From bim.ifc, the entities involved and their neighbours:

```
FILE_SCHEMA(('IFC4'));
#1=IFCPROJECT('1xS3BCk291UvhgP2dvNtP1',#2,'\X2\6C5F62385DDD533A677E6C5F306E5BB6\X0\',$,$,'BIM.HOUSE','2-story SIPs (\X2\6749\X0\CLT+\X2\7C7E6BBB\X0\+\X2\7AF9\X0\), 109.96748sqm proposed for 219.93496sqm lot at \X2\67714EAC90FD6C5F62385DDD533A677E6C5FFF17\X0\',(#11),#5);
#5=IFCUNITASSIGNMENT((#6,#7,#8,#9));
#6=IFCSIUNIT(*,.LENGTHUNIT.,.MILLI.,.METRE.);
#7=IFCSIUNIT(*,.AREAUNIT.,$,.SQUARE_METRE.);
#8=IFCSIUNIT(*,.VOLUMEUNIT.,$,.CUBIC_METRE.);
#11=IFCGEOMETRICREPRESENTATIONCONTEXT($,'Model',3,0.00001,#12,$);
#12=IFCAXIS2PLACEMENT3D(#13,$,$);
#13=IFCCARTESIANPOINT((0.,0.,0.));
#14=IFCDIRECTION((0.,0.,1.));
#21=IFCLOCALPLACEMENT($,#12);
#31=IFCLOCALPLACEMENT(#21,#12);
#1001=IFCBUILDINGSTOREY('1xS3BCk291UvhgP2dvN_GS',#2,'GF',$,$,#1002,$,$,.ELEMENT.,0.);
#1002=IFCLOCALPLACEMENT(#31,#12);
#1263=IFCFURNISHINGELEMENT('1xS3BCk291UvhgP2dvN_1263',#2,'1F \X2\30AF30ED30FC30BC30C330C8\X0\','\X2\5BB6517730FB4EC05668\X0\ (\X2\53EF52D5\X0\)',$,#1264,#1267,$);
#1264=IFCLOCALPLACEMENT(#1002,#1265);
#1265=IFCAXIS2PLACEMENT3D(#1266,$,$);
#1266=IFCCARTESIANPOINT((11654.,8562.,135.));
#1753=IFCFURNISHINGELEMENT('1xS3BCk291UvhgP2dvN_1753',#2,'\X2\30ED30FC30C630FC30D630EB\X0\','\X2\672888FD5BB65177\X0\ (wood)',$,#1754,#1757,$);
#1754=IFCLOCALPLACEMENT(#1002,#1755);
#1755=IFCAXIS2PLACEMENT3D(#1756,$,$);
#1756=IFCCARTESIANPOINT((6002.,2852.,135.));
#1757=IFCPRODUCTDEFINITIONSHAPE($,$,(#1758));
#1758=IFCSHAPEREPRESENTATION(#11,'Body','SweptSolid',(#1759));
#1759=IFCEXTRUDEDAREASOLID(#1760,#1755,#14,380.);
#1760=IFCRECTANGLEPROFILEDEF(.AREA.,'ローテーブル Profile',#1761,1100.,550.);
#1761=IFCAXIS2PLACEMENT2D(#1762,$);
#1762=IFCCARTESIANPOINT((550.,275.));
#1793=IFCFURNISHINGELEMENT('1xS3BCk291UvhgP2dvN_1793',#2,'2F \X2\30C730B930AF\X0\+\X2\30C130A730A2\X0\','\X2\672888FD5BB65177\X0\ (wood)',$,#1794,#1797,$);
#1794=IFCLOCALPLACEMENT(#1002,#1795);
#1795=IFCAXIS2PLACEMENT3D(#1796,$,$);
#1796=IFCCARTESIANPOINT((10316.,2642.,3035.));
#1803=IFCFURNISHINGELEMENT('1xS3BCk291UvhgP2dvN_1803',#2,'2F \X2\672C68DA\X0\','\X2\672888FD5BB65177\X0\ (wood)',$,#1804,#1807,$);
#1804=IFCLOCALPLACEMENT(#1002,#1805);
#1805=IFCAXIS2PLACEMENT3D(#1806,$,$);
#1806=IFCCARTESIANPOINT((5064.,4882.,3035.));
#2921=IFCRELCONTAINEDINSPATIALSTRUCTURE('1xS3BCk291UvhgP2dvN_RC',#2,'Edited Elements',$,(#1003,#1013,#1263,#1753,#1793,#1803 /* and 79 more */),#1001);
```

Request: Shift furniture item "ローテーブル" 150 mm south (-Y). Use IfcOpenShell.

```python
import ifcopenshell
import ifcopenshell.api.geometry
import ifcopenshell.util.placement
import ifcopenshell.util.unit

model = ifcopenshell.open("bim.ifc")
unit_scale = ifcopenshell.util.unit.calculate_unit_scale(model)

item = model.by_id(1753)
matrix = ifcopenshell.util.placement.get_local_placement(item.ObjectPlacement)
matrix[1, 3] -= 0.15 / unit_scale
ifcopenshell.api.geometry.edit_object_placement(model, product=item, matrix=matrix, is_si=False)

print(ifcopenshell.util.placement.get_local_placement(item.ObjectPlacement).round(3) + 0.0)

model.write("bim_rev.ifc")
```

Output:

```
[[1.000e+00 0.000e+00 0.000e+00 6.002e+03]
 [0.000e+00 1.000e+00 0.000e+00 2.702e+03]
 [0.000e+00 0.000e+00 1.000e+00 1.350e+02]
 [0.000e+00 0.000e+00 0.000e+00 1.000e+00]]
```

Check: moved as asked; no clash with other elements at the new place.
